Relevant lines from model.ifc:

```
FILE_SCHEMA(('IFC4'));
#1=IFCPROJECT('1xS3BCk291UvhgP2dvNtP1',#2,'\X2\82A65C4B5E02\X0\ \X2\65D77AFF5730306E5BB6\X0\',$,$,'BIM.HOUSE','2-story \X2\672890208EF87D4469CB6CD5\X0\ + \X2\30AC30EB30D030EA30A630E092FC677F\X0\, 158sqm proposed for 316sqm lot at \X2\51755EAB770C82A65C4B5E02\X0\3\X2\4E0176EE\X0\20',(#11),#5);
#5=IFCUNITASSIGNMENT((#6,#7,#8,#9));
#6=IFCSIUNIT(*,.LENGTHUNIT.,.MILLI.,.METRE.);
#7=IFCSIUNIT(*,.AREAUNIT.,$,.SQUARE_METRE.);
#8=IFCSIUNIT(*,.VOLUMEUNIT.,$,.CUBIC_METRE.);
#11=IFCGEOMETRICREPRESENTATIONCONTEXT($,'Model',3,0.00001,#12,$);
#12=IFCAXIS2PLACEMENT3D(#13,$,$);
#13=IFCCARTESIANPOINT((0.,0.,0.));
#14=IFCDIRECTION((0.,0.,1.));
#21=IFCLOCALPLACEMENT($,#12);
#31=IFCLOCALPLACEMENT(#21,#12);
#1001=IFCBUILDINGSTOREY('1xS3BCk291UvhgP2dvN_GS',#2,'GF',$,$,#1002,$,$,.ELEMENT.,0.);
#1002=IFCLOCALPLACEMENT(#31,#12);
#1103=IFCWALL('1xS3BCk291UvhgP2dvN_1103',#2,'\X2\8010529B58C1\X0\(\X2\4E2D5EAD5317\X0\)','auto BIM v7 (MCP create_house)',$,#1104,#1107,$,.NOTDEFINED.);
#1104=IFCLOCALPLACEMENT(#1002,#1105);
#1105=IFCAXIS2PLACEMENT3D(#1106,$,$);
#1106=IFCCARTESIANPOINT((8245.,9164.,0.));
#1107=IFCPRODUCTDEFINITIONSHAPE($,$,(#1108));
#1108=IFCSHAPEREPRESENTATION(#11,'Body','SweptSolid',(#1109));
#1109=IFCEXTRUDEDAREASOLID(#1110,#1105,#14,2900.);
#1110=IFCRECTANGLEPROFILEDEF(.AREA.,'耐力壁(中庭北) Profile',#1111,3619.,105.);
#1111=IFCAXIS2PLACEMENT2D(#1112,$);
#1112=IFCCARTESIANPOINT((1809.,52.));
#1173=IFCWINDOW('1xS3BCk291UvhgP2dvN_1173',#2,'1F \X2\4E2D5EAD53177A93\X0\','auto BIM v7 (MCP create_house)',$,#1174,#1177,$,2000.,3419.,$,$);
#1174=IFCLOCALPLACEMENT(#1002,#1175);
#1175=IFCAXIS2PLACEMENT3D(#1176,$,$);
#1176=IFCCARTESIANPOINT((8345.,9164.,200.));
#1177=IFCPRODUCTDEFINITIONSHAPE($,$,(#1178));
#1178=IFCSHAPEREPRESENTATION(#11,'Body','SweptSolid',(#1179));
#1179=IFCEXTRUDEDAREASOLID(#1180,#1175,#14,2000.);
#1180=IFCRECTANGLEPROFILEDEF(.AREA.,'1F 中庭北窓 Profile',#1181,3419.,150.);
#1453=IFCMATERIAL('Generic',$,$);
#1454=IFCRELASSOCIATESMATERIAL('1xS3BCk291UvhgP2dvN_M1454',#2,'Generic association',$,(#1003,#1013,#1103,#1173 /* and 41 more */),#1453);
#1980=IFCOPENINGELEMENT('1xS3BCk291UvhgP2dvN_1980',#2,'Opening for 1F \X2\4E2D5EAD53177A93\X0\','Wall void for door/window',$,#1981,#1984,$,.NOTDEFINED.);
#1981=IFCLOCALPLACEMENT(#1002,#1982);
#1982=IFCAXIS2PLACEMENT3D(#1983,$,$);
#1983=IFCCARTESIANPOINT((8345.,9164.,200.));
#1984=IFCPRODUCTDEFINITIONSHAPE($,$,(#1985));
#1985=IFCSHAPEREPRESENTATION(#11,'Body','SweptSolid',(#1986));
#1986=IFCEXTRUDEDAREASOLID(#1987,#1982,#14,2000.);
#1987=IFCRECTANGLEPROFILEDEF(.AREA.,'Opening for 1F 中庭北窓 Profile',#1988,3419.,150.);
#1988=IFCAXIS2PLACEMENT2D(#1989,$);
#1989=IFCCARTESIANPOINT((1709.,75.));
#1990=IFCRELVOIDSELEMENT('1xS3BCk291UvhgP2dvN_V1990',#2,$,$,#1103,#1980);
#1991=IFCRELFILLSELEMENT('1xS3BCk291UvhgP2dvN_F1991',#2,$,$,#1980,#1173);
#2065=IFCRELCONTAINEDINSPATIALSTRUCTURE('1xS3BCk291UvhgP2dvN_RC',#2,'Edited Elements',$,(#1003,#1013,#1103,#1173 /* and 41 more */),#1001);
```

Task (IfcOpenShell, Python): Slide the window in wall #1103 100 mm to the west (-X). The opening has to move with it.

```python
import ifcopenshell
import ifcopenshell.api.geometry
import ifcopenshell.util.placement
import ifcopenshell.util.unit

model = ifcopenshell.open("model.ifc")
unit_scale = ifcopenshell.util.unit.calculate_unit_scale(model)

window = model.by_guid("1xS3BCk291UvhgP2dvN_1173")
opening = window.FillsVoids[0].RelatingOpeningElement
wall = opening.VoidsElements[0].RelatingBuildingElement

wall_matrix = ifcopenshell.util.placement.get_local_placement(wall.ObjectPlacement)
shift = wall_matrix[:3, 0] * -0.1 / unit_scale
before = ifcopenshell.util.placement.get_local_placement(window.ObjectPlacement)[:3, 3].copy()

# The window is not placed relative to its opening, so move both.
for product in (opening, window):
    matrix = ifcopenshell.util.placement.get_local_placement(product.ObjectPlacement)
    matrix[:3, 3] += shift
    ifcopenshell.api.geometry.edit_object_placement(model, product=product, matrix=matrix, is_si=False)

after = ifcopenshell.util.placement.get_local_placement(window.ObjectPlacement)[:3, 3]
print("window moved by", (after - before).round(3) + 0.0)

model.write("model-out.ifc")
```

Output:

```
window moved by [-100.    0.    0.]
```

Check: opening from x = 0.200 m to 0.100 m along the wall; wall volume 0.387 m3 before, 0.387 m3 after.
